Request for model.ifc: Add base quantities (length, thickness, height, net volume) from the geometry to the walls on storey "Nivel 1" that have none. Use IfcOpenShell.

First a look at what the model holds.

```python
import ifcopenshell
import ifcopenshell.util.element
import ifcopenshell.util.unit

model = ifcopenshell.open("model.ifc")
print(model.schema)
for unit_type in ("LENGTHUNIT", "AREAUNIT", "VOLUMEUNIT"):
    print(unit_type, ifcopenshell.util.unit.calculate_unit_scale(model, unit_type))
storey = next(s for s in model.by_type("IfcBuildingStorey") if s.Name == "Nivel 1")
walls = [e for e in ifcopenshell.util.element.get_decomposition(storey) if e.is_a("IfcWall")]
for e in sorted(walls, key=lambda e: e.id()):
    print(e.id(), e.is_a(), e.Name, list(ifcopenshell.util.element.get_psets(e, qtos_only=True)), sep=" | ")
```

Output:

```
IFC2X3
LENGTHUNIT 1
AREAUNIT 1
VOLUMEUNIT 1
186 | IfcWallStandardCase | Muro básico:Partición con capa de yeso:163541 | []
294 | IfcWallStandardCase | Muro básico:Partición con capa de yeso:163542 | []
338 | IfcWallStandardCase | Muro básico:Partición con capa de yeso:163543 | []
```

```python
import ifcopenshell
import ifcopenshell.api.pset
import ifcopenshell.geom
import ifcopenshell.util.element
import ifcopenshell.util.shape
import ifcopenshell.util.unit

model = ifcopenshell.open("model.ifc")
unit_scale = ifcopenshell.util.unit.calculate_unit_scale(model)
volume_scale = ifcopenshell.util.unit.calculate_unit_scale(model, "VOLUMEUNIT")
settings = ifcopenshell.geom.settings()

storey = next(s for s in model.by_type("IfcBuildingStorey") if s.Name == "Nivel 1")
walls = [e for e in ifcopenshell.util.element.get_decomposition(storey) if e.is_a("IfcWall")]

for e in sorted(walls, key=lambda e: e.id()):
    if ifcopenshell.util.element.get_psets(e, qtos_only=True, should_inherit=False):
        continue
    # Geometry comes back in metres, in the element's own axes.
    shape = ifcopenshell.geom.create_shape(settings, e)
    values = {
        "Length": ifcopenshell.util.shape.get_x(shape.geometry) / unit_scale,
        "Width": ifcopenshell.util.shape.get_y(shape.geometry) / unit_scale,
        "Height": ifcopenshell.util.shape.get_z(shape.geometry) / unit_scale,
        "NetVolume": ifcopenshell.util.shape.get_volume(shape.geometry) / volume_scale,
    }
    qto = ifcopenshell.api.pset.add_qto(model, product=e, name="BaseQuantities")
    ifcopenshell.api.pset.edit_qto(model, qto=qto, properties=values)
    print(e.id(), {k: round(v, 3) for k, v in values.items()})

model.write("model-out.ifc")
```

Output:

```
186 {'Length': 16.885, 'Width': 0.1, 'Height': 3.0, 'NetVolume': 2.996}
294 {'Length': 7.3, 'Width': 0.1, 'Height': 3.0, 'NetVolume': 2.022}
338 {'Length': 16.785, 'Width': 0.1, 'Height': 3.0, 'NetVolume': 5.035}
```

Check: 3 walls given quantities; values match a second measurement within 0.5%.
